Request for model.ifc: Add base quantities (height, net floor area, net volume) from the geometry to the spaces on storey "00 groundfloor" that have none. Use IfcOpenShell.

First a look at what the model holds.

```python
import ifcopenshell
import ifcopenshell.util.element
import ifcopenshell.util.unit

model = ifcopenshell.open("model.ifc")
print(model.schema)
for unit_type in ("LENGTHUNIT", "AREAUNIT", "VOLUMEUNIT"):
    print(unit_type, ifcopenshell.util.unit.calculate_unit_scale(model, unit_type))
storey = next(s for s in model.by_type("IfcBuildingStorey") if s.Name == "00 groundfloor")
spaces = [e for e in ifcopenshell.util.element.get_decomposition(storey) if e.is_a("IfcSpace")]
for e in sorted(spaces, key=lambda e: e.id()):
    print(e.id(), e.is_a(), e.Name, list(ifcopenshell.util.element.get_psets(e, qtos_only=True)), sep=" | ")
```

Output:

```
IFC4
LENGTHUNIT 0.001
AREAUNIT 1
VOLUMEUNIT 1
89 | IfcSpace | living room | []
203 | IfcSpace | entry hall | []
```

```python
import ifcopenshell
import ifcopenshell.api.pset
import ifcopenshell.geom
import ifcopenshell.util.element
import ifcopenshell.util.shape
import ifcopenshell.util.unit

model = ifcopenshell.open("model.ifc")
unit_scale = ifcopenshell.util.unit.calculate_unit_scale(model)
area_scale = ifcopenshell.util.unit.calculate_unit_scale(model, "AREAUNIT")
volume_scale = ifcopenshell.util.unit.calculate_unit_scale(model, "VOLUMEUNIT")
settings = ifcopenshell.geom.settings()

storey = next(s for s in model.by_type("IfcBuildingStorey") if s.Name == "00 groundfloor")
spaces = [e for e in ifcopenshell.util.element.get_decomposition(storey) if e.is_a("IfcSpace")]

for e in sorted(spaces, key=lambda e: e.id()):
    if ifcopenshell.util.element.get_psets(e, qtos_only=True, should_inherit=False):
        continue
    # Geometry comes back in metres, in the element's own axes.
    shape = ifcopenshell.geom.create_shape(settings, e)
    values = {
        "Height": ifcopenshell.util.shape.get_z(shape.geometry) / unit_scale,
        "NetFloorArea": ifcopenshell.util.shape.get_footprint_area(shape.geometry) / area_scale,
        "NetVolume": ifcopenshell.util.shape.get_volume(shape.geometry) / volume_scale,
    }
    qto = ifcopenshell.api.pset.add_qto(model, product=e, name="Qto_SpaceBaseQuantities")
    ifcopenshell.api.pset.edit_qto(model, qto=qto, properties=values)
    print(e.id(), {k: round(v, 3) for k, v in values.items()})

model.write("model_rev.ifc")
```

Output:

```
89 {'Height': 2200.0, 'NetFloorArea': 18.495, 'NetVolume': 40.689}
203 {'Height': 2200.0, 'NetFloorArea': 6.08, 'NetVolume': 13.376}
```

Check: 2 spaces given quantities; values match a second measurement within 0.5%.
